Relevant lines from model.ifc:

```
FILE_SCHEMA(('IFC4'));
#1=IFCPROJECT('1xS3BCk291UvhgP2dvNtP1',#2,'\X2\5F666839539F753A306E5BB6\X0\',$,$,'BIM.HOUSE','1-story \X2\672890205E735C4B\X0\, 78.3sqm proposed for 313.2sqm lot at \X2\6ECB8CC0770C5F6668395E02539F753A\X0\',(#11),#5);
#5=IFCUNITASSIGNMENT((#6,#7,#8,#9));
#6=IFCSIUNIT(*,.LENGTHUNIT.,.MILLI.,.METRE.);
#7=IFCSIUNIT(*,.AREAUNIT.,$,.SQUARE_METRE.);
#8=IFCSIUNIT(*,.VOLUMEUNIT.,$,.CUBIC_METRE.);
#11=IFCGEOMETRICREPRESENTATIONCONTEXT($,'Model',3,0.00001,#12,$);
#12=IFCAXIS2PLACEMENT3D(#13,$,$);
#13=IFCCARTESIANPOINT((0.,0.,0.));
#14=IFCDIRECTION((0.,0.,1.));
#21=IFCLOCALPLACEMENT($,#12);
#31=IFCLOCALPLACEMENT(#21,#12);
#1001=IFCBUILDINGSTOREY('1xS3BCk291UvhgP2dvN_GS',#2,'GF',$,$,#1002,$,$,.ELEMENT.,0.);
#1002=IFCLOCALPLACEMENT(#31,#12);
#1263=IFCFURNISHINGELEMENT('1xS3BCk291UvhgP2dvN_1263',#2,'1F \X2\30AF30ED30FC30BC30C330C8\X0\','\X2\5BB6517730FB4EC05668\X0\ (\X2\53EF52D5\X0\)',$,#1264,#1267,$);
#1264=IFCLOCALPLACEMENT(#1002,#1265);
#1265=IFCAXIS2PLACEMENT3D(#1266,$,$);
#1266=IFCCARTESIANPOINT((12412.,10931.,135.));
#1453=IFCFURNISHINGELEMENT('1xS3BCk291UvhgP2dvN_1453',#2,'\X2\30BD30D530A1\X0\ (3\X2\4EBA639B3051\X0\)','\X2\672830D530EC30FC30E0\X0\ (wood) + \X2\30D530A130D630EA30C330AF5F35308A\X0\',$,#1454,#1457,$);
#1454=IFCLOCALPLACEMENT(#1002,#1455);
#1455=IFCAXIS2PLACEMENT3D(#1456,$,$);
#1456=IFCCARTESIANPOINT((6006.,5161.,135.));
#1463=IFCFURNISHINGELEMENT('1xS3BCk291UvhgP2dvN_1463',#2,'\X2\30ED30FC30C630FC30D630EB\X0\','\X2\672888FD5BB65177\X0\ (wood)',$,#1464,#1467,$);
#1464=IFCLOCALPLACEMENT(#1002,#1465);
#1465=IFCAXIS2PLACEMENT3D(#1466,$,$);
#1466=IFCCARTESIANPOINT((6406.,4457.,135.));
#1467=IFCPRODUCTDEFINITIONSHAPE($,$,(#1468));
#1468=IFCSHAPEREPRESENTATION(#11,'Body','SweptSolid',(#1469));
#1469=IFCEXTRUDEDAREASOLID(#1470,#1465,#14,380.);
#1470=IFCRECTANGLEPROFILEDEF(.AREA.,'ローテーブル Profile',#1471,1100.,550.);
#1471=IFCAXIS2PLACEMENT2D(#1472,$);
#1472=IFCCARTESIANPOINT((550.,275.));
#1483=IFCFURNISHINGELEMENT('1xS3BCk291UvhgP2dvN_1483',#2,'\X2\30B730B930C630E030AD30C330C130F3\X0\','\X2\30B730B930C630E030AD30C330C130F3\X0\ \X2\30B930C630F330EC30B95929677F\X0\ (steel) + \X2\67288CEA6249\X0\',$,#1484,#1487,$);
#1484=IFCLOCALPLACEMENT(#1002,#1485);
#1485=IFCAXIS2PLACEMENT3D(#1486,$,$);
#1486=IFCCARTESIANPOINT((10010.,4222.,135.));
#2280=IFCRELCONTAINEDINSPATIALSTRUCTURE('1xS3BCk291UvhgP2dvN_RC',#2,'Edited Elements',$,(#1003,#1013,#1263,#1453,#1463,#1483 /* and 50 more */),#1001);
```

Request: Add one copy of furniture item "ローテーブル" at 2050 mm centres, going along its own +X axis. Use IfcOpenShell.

```python
import ifcopenshell
import ifcopenshell.api.geometry
import ifcopenshell.api.root
import ifcopenshell.util.element
import ifcopenshell.util.placement

model = ifcopenshell.open("model.ifc")


def reuse_history(source, copy):
    """copy_class also copies each property set's owner history, people and application; keep the originals."""
    for rel in copy.IsDefinedBy:
        if rel.is_a("IfcRelDefinesByProperties") and (history := rel.RelatingPropertyDefinition.OwnerHistory):
            rel.RelatingPropertyDefinition.OwnerHistory = source.OwnerHistory
            ifcopenshell.util.element.remove_deep2(model, history)


source = model.by_guid("1xS3BCk291UvhgP2dvN_1463")
base = ifcopenshell.util.placement.get_local_placement(source.ObjectPlacement)
step = base[:3, 0] * 2050.0

for i in range(1, 2):
    copy = ifcopenshell.api.root.copy_class(model, product=source)
    copy.Representation = ifcopenshell.util.element.copy_deep(
        model, source.Representation, exclude=["IfcGeometricRepresentationContext", "IfcRepresentationMap"]
    )
    reuse_history(source, copy)
    matrix = base.copy()
    matrix[:3, 3] += i * step
    print("added at", matrix[:3, 3].round(3) + 0.0)
    ifcopenshell.api.geometry.edit_object_placement(model, product=copy, matrix=matrix, is_si=False)

model.write("model_rev.ifc")
```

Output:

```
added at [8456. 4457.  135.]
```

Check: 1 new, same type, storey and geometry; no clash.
